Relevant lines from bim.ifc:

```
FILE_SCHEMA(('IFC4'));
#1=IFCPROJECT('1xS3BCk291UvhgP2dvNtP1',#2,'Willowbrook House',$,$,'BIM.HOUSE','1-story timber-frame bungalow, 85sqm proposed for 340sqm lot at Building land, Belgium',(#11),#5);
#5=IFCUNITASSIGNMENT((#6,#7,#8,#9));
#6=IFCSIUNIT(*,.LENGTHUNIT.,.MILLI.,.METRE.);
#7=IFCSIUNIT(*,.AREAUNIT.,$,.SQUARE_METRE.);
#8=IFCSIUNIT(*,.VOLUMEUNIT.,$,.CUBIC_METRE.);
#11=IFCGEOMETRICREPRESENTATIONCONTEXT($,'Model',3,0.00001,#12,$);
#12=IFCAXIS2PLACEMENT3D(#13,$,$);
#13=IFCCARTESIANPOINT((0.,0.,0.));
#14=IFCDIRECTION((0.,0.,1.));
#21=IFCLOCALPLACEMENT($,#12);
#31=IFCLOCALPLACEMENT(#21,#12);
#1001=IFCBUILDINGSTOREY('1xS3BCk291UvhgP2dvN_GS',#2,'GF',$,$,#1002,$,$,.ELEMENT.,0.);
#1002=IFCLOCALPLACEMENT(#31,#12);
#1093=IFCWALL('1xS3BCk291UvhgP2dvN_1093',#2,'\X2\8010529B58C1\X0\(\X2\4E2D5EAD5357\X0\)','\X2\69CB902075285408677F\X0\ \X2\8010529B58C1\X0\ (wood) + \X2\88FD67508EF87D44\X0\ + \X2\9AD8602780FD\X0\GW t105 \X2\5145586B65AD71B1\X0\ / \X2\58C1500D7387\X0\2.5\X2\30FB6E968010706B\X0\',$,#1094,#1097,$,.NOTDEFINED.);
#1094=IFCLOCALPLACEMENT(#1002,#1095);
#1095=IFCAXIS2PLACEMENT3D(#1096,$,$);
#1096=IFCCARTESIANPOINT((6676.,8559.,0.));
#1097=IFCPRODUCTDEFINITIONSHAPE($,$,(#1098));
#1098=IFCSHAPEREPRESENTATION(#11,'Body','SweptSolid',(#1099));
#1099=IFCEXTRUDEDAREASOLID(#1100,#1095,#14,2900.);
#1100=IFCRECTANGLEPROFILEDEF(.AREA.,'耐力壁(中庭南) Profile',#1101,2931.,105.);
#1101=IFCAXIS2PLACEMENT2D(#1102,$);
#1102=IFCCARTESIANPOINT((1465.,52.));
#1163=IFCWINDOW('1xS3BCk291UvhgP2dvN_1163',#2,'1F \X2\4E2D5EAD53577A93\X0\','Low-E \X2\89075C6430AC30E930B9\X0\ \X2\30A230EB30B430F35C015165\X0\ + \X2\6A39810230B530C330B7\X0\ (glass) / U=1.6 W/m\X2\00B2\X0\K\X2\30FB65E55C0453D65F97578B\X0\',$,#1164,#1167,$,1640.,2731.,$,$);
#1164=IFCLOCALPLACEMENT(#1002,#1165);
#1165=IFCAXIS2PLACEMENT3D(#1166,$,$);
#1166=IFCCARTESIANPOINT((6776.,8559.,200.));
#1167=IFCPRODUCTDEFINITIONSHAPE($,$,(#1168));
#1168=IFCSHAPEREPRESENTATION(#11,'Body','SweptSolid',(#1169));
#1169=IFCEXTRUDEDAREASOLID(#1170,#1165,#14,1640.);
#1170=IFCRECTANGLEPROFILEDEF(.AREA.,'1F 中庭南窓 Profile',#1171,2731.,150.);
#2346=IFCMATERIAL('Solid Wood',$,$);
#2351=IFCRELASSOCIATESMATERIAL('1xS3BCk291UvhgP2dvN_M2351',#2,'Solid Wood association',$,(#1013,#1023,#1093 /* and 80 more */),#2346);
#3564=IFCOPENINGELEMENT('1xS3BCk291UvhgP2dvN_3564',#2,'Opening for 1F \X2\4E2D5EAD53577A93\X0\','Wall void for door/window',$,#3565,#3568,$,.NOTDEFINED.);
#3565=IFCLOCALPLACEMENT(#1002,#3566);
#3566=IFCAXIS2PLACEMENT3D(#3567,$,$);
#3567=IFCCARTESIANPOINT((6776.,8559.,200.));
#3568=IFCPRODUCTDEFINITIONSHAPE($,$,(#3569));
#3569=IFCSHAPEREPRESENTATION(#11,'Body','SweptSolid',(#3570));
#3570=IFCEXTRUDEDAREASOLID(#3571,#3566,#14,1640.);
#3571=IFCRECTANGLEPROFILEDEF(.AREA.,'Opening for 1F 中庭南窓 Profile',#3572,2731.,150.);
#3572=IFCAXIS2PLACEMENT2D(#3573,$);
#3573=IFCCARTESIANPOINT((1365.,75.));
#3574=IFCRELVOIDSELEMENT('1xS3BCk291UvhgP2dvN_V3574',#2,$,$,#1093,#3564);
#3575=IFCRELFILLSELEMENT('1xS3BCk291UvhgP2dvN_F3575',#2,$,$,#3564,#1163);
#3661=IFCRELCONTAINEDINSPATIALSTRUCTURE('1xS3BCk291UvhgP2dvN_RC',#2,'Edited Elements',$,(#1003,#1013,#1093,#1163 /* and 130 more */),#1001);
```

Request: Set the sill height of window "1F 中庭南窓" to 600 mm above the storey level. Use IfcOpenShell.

```python
import numpy as np
import ifcopenshell
import ifcopenshell.api.geometry
import ifcopenshell.geom
import ifcopenshell.util.element
import ifcopenshell.util.placement
import ifcopenshell.util.shape
import ifcopenshell.util.unit

model = ifcopenshell.open("bim.ifc")
unit_scale = ifcopenshell.util.unit.calculate_unit_scale(model)

window = model.by_guid("1xS3BCk291UvhgP2dvN_1163")
opening = window.FillsVoids[0].RelatingOpeningElement
storey = ifcopenshell.util.element.get_container(window, ifc_class="IfcBuildingStorey")
level = ifcopenshell.util.placement.get_local_placement(storey.ObjectPlacement)[2, 3]

# The opening's origin need not be at the sill, so measure its lowest point.
shape = ifcopenshell.geom.create_shape(ifcopenshell.geom.settings(), opening)
bottom = ifcopenshell.util.shape.get_shape_bottom_elevation(shape, shape.geometry) / unit_scale
dz = level + 600.0 - bottom

shift = np.array([0.0, 0.0, dz])
# The window is not placed relative to its opening, so move both.
for product in (opening, window):
    matrix = ifcopenshell.util.placement.get_local_placement(product.ObjectPlacement)
    matrix[:3, 3] += shift
    ifcopenshell.api.geometry.edit_object_placement(model, product=product, matrix=matrix, is_si=False)

print(f"moved by {dz * unit_scale:+.3f} m")

model.write("bim_edited.ifc")
```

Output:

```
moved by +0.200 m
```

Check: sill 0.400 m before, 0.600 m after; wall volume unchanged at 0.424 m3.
